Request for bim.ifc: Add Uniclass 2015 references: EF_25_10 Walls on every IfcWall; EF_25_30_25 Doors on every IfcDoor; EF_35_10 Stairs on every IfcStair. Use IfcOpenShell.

First a look at what the model holds.

```python
import ifcopenshell

model = ifcopenshell.open("bim.ifc")
print(model.schema)
print("classifications:", [c.Name for c in model.by_type("IfcClassification")])
for ifc_class in ("IfcDoor", "IfcRoof", "IfcStair", "IfcWall", "IfcWindow"):
    print(ifc_class, len(model.by_type(ifc_class)))
```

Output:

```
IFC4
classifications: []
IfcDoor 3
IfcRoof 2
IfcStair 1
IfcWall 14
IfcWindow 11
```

```python
import ifcopenshell
import ifcopenshell.api.classification

model = ifcopenshell.open("bim.ifc")

system = ifcopenshell.api.classification.add_classification(model, classification="Uniclass 2015")

codes = {
    "IfcWall": ("EF_25_10", "Walls"),
    "IfcDoor": ("EF_25_30_25", "Doors"),
    "IfcStair": ("EF_35_10", "Stairs"),
}
for ifc_class, (code, name) in codes.items():
    products = model.by_type(ifc_class)
    ifcopenshell.api.classification.add_reference(
        model, products=products, classification=system, identification=code, name=name
    )
    print(code, len(products))

model.write("bim_rev.ifc")
```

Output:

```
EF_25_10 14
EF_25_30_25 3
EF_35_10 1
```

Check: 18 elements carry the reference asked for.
